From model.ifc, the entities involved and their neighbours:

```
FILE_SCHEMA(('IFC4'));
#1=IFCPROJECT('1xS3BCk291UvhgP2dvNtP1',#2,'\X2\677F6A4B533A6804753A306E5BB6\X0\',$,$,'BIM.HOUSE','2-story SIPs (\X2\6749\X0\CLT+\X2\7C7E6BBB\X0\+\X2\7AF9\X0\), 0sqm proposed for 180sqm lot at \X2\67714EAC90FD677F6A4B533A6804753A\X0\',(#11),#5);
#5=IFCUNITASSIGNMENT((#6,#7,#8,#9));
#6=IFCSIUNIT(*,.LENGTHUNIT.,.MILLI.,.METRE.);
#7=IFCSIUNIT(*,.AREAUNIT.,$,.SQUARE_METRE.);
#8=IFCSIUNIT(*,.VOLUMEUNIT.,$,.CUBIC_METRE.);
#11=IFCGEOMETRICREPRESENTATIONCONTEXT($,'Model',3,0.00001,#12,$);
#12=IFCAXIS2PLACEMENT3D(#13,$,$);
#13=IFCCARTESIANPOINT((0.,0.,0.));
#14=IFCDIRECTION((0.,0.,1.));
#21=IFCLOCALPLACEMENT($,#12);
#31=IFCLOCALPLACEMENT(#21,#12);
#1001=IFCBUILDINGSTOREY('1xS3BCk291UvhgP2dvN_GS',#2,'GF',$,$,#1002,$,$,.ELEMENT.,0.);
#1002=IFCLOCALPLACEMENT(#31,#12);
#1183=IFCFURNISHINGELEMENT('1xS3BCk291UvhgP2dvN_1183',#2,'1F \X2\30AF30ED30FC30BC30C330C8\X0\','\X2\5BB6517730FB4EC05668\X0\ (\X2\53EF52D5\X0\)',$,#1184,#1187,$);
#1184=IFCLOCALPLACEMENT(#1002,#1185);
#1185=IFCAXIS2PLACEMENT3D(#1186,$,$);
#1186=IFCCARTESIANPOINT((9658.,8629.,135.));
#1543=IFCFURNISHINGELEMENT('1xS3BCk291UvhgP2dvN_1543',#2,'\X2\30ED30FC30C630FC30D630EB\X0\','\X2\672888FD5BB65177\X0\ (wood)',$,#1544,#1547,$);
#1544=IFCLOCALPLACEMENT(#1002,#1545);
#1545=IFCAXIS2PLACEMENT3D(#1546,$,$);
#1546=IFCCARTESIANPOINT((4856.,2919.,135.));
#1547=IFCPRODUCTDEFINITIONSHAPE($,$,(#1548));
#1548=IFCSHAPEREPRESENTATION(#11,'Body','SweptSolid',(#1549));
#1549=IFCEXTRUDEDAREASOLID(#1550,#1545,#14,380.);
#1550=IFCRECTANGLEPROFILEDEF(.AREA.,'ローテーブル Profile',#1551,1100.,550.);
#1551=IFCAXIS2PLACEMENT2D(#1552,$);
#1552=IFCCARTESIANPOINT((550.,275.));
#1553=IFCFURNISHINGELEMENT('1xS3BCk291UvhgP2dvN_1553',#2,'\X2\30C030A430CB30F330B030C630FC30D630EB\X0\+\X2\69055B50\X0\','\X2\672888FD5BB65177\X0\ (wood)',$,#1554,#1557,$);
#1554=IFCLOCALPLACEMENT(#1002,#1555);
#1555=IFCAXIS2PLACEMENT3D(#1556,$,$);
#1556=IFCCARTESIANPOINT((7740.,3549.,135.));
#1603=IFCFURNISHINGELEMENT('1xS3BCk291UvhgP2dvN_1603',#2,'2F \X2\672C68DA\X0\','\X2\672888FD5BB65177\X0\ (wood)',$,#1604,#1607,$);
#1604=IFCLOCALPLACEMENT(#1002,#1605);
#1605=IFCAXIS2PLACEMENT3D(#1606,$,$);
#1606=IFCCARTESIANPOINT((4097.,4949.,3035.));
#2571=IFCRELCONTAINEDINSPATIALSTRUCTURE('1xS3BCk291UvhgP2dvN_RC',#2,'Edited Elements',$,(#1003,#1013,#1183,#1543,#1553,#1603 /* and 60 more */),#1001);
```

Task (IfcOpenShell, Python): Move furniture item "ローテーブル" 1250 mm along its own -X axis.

```python
import ifcopenshell
import ifcopenshell.api.geometry
import ifcopenshell.util.placement

model = ifcopenshell.open("model.ifc")

item = model.by_guid("1xS3BCk291UvhgP2dvN_1543")
matrix = ifcopenshell.util.placement.get_local_placement(item.ObjectPlacement)
matrix[:3, 3] -= matrix[:3, 0] * 1250.0
ifcopenshell.api.geometry.edit_object_placement(model, product=item, matrix=matrix, is_si=False)

print(ifcopenshell.util.placement.get_local_placement(item.ObjectPlacement).round(3) + 0.0)

model.write("model_edited.ifc")
```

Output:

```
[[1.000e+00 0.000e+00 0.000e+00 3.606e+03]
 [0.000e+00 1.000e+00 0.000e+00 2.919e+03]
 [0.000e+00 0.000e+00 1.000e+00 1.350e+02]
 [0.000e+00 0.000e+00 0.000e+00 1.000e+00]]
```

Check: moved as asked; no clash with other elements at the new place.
